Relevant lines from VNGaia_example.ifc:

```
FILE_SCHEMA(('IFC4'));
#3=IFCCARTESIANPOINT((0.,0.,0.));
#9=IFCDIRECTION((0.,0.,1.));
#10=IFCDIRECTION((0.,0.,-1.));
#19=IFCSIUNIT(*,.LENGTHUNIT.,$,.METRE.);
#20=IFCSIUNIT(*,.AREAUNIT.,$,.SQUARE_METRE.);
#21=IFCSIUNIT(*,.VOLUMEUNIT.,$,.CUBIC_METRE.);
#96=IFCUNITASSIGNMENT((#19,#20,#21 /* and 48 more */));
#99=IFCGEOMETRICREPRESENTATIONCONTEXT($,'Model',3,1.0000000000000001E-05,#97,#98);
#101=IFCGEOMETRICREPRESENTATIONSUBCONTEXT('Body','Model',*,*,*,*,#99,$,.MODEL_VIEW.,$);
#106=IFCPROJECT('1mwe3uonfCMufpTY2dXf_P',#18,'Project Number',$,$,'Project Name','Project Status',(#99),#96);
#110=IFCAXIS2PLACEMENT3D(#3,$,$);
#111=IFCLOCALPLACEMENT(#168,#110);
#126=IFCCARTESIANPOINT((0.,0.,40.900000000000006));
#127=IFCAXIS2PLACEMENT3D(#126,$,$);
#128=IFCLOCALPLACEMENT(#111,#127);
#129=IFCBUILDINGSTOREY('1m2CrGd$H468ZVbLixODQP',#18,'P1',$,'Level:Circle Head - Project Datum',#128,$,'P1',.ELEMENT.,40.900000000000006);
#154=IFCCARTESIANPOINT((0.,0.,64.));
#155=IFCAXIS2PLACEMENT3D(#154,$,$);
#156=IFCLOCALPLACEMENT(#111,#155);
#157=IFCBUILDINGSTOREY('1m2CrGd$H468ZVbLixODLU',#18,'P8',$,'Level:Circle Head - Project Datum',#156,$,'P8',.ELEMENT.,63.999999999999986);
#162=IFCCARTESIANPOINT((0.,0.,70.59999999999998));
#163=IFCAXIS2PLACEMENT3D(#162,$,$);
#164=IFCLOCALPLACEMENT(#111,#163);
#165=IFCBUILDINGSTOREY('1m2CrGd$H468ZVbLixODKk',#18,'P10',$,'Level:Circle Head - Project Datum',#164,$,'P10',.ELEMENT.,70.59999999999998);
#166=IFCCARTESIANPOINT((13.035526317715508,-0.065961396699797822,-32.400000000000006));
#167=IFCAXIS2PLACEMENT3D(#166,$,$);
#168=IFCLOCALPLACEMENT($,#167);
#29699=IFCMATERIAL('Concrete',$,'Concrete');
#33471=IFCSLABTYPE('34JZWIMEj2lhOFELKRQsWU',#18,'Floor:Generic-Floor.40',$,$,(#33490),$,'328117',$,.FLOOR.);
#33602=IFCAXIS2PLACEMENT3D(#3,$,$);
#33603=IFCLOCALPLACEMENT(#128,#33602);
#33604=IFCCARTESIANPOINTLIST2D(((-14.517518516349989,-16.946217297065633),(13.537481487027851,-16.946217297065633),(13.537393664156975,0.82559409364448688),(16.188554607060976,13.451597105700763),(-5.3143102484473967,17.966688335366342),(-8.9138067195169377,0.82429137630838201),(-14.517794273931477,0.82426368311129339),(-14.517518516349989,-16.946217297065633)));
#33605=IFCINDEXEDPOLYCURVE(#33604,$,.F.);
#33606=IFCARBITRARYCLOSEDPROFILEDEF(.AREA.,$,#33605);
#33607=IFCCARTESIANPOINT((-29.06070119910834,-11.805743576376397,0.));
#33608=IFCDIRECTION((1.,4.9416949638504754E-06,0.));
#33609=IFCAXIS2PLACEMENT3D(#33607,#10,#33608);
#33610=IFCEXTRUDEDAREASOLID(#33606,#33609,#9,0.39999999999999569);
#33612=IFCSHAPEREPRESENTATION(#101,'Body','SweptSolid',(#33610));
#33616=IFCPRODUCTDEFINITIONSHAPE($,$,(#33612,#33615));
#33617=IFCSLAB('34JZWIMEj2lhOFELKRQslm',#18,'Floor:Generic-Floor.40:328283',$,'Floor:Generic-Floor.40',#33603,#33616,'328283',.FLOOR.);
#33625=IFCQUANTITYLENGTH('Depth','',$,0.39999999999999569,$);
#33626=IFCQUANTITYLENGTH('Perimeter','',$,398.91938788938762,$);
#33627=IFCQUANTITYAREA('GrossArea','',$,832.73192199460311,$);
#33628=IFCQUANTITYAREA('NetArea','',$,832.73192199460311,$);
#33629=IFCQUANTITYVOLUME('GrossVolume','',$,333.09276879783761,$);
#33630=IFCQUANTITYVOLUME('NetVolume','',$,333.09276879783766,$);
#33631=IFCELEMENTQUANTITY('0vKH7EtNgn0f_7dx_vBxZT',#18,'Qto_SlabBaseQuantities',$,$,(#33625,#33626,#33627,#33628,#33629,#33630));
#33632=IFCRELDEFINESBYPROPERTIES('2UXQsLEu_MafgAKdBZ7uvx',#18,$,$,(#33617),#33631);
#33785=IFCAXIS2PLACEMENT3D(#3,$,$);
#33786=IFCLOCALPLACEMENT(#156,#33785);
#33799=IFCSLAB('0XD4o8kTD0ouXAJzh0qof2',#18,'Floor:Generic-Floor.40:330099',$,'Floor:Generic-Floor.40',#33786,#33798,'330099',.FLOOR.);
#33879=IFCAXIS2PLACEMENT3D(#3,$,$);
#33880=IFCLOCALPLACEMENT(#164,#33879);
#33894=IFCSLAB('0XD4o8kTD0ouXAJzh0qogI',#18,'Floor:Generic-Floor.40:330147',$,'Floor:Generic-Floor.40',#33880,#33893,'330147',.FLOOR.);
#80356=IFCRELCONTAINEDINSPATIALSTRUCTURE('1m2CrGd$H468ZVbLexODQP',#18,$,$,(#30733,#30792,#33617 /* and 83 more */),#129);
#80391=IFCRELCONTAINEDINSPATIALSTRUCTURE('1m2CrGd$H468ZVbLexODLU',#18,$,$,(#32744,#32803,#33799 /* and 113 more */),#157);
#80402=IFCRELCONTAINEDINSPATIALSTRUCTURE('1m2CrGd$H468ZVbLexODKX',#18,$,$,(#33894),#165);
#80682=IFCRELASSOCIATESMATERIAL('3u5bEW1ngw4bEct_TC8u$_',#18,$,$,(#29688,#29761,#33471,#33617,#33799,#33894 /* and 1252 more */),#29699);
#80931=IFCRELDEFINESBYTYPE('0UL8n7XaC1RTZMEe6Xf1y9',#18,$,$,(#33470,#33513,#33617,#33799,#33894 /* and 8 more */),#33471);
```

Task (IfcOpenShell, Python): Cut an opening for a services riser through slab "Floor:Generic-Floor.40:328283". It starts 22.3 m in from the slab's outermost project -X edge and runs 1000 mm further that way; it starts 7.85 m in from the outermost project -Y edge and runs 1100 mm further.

```python
import numpy as np
import ifcopenshell
import ifcopenshell.api.feature
import ifcopenshell.api.geometry
import ifcopenshell.api.pset
import ifcopenshell.api.root
import ifcopenshell.geom
import ifcopenshell.util.element
import ifcopenshell.util.placement
import ifcopenshell.util.representation
import ifcopenshell.util.shape
import ifcopenshell.util.unit

model = ifcopenshell.open("VNGaia_example.ifc")
unit_scale = ifcopenshell.util.unit.calculate_unit_scale(model)
area_scale = ifcopenshell.util.unit.calculate_unit_scale(model, "AREAUNIT")
volume_scale = ifcopenshell.util.unit.calculate_unit_scale(model, "VOLUMEUNIT")
settings = ifcopenshell.geom.settings()


def volume(element):
    """Net volume in cubic metres, openings subtracted."""
    shape = ifcopenshell.geom.create_shape(settings, element)
    return ifcopenshell.util.shape.get_volume(shape.geometry)


slab = model.by_guid("34JZWIMEj2lhOFELKRQslm")
before = volume(slab)

# Extent in the slab's own axes, in metres. The edges named are its -X and -Y sides.
slab_shape = ifcopenshell.geom.create_shape(settings, slab)
vertices = ifcopenshell.util.shape.get_vertices(slab_shape.geometry)
x_min, y_min, bottom = vertices.min(axis=0)
top = vertices[:, 2].max()

opening = ifcopenshell.api.root.create_entity(model, ifc_class="IfcOpeningElement", name="Services riser opening", predefined_type="OPENING")
context = ifcopenshell.util.representation.get_context(model, "Model", "Body", "MODEL_VIEW")
width, depth = 1, 1.1
outline = [(0.0, 0.0), (width, 0.0), (width, depth), (0.0, depth), (0.0, 0.0)]
# Overshoot both faces by 50 mm so the cut is clean.
shape = ifcopenshell.api.geometry.add_slab_representation(
    model, context=context, depth=top - bottom + 0.1, polyline=outline
)
ifcopenshell.api.geometry.assign_representation(model, product=opening, representation=shape)

matrix = ifcopenshell.util.placement.get_local_placement(slab.ObjectPlacement)
matrix[:, 3] = matrix @ np.append(np.array([x_min + 22.3, y_min + 7.85, bottom - 0.05]) / unit_scale, 1.0)
ifcopenshell.api.geometry.edit_object_placement(model, product=opening, matrix=matrix, is_si=False)
ifcopenshell.api.feature.add_feature(model, feature=opening, element=slab)

after = volume(slab)

# Update the slab's stored quantities.
qto = model.by_id(ifcopenshell.util.element.get_pset(slab, "Qto_SlabBaseQuantities", should_inherit=False)["id"])
ifcopenshell.api.pset.edit_qto(model, qto=qto, properties={
    "NetArea": after / (top - bottom) / area_scale,
    "NetVolume": after / volume_scale,
})

print(f"slab volume {before:.3f} -> {after:.3f} m3")

model.write("VNGaia_example_edited.ifc")
```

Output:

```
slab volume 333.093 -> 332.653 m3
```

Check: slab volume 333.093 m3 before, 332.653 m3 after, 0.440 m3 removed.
